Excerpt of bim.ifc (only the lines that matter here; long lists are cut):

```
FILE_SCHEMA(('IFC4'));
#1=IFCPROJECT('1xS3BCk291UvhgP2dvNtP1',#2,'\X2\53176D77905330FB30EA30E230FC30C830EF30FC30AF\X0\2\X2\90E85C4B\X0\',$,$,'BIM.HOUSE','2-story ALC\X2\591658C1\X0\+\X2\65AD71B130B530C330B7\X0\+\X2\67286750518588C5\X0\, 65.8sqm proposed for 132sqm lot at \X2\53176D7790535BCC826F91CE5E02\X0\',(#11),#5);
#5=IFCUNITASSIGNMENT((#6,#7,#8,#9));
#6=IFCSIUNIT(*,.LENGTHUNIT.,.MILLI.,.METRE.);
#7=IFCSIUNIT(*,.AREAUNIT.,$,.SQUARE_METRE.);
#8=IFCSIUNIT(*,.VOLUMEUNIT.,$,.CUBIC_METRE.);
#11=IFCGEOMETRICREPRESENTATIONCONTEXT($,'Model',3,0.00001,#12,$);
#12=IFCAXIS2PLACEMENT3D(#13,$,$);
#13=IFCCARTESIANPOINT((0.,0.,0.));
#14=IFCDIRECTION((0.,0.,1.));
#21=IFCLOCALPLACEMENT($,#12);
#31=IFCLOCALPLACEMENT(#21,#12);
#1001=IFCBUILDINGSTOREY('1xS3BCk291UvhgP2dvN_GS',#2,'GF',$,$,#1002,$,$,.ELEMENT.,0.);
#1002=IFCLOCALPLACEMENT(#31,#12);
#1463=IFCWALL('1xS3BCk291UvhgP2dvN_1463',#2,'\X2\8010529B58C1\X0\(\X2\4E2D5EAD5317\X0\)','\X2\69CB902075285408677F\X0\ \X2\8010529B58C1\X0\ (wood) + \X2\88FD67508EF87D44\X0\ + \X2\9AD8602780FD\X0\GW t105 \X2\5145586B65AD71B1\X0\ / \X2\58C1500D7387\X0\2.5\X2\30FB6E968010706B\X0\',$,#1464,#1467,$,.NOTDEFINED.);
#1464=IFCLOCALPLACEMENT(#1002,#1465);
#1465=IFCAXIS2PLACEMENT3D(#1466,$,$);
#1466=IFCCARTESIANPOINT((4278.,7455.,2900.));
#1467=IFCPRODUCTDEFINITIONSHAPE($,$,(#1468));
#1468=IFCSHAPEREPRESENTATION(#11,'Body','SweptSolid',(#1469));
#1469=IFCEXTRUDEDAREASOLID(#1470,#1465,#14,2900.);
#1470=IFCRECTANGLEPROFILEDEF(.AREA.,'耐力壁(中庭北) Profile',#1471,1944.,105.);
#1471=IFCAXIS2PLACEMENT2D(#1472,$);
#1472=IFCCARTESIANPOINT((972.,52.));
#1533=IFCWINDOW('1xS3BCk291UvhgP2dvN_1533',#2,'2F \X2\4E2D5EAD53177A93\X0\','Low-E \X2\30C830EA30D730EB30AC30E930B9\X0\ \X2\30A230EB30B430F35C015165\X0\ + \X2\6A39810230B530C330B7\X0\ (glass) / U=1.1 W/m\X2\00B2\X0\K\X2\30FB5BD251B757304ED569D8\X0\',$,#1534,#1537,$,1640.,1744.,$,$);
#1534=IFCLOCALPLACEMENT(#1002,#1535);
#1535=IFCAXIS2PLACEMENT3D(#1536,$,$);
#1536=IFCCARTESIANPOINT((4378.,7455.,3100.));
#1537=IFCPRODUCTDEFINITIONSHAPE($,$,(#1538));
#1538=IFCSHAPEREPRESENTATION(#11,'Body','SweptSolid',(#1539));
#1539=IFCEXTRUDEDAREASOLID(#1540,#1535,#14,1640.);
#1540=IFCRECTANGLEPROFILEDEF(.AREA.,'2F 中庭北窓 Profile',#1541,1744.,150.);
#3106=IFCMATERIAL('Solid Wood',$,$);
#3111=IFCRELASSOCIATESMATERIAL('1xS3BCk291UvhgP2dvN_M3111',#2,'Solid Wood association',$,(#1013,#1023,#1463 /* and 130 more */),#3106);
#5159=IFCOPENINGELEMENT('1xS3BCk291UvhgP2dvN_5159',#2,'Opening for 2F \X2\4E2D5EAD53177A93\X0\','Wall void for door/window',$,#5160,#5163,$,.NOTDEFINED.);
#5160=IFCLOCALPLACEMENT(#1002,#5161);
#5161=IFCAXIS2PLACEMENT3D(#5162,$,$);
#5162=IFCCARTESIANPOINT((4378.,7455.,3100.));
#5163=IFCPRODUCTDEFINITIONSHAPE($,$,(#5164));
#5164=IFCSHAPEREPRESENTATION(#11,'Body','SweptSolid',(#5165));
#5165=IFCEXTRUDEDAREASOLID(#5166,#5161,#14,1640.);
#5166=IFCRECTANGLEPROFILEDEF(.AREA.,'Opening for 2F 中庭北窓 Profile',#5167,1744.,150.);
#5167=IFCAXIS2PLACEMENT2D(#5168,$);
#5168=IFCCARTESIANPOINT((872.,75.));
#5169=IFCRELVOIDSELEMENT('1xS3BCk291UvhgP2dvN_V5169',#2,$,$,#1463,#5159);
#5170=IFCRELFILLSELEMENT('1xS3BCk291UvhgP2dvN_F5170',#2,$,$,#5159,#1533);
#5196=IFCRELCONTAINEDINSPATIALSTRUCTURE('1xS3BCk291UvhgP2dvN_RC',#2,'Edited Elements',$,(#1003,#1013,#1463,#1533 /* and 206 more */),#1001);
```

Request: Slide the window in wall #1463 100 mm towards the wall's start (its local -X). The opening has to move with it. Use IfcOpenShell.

```python
import ifcopenshell
import ifcopenshell.api.geometry
import ifcopenshell.util.placement

model = ifcopenshell.open("bim.ifc")

window = model.by_id(1533)
opening = window.FillsVoids[0].RelatingOpeningElement
wall = opening.VoidsElements[0].RelatingBuildingElement

wall_matrix = ifcopenshell.util.placement.get_local_placement(wall.ObjectPlacement)
shift = wall_matrix[:3, 0] * -100.0
before = ifcopenshell.util.placement.get_local_placement(window.ObjectPlacement)[:3, 3].copy()

# The window is not placed relative to its opening, so move both.
for product in (opening, window):
    matrix = ifcopenshell.util.placement.get_local_placement(product.ObjectPlacement)
    matrix[:3, 3] += shift
    ifcopenshell.api.geometry.edit_object_placement(model, product=product, matrix=matrix, is_si=False)

after = ifcopenshell.util.placement.get_local_placement(window.ObjectPlacement)[:3, 3]
print("window moved by", (after - before).round(3) + 0.0)

model.write("bim_updated.ifc")
```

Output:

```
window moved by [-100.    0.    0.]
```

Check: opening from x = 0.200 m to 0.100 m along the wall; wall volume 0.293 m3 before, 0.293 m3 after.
